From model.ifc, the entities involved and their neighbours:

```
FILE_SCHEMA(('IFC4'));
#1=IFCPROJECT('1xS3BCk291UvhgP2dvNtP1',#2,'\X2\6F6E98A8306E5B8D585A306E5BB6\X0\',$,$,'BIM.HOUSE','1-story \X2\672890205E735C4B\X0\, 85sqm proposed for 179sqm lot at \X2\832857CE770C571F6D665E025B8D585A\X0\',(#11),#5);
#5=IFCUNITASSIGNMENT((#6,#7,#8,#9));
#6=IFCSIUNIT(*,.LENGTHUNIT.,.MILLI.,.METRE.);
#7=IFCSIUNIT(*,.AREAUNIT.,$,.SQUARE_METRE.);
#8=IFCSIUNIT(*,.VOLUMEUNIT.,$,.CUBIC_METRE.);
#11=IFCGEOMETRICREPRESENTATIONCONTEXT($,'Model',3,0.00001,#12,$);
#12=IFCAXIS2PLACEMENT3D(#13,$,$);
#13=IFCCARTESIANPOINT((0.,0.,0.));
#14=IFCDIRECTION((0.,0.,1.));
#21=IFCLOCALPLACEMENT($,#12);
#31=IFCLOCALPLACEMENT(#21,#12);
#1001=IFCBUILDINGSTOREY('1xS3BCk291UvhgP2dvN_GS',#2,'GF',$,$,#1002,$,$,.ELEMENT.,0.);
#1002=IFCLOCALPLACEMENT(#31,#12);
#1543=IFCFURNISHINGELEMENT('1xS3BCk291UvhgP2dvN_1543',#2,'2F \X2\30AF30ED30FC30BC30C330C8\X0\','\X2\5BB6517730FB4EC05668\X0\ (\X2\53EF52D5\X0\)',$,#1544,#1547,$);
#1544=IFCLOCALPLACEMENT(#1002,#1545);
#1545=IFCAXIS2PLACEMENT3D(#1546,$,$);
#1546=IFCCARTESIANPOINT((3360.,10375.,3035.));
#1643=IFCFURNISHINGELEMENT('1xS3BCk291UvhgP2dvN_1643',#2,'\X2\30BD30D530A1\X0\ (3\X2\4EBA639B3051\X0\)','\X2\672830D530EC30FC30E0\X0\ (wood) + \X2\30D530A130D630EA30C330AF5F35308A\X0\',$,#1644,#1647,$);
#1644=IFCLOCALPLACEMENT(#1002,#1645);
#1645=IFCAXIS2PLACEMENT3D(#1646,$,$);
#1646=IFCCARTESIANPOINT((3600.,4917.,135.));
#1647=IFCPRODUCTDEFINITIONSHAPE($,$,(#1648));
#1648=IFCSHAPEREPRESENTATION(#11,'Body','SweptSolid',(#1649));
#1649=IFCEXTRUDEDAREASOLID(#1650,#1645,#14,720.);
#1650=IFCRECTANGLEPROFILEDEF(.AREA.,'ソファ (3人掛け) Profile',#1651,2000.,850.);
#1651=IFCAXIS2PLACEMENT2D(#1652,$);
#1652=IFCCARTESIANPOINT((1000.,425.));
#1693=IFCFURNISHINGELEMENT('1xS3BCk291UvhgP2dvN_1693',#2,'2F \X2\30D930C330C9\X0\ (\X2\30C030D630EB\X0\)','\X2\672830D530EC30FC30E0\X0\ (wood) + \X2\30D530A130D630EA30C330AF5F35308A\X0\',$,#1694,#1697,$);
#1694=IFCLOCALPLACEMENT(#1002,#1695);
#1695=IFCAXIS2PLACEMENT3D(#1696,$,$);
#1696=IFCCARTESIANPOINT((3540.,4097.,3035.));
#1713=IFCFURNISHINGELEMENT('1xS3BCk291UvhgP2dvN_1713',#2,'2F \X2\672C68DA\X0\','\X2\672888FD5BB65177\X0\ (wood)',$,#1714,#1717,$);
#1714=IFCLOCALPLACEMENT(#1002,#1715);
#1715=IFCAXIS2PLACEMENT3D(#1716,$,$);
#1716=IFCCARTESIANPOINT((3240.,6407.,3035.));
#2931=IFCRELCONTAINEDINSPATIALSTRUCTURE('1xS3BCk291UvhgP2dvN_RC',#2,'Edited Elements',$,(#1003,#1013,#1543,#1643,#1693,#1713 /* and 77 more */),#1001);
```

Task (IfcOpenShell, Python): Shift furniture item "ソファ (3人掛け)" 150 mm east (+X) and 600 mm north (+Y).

```python
import ifcopenshell
import ifcopenshell.api.geometry
import ifcopenshell.util.placement
import ifcopenshell.util.unit

model = ifcopenshell.open("model.ifc")
unit_scale = ifcopenshell.util.unit.calculate_unit_scale(model)

item = model.by_guid("1xS3BCk291UvhgP2dvN_1643")
matrix = ifcopenshell.util.placement.get_local_placement(item.ObjectPlacement)
matrix[0, 3] += 0.15 / unit_scale
matrix[1, 3] += 0.6 / unit_scale
ifcopenshell.api.geometry.edit_object_placement(model, product=item, matrix=matrix, is_si=False)

print(ifcopenshell.util.placement.get_local_placement(item.ObjectPlacement).round(3) + 0.0)

model.write("model-out.ifc")
```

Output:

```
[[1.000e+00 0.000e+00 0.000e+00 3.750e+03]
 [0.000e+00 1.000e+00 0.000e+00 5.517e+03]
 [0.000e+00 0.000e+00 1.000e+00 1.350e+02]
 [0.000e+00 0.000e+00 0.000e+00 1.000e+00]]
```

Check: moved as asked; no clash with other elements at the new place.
